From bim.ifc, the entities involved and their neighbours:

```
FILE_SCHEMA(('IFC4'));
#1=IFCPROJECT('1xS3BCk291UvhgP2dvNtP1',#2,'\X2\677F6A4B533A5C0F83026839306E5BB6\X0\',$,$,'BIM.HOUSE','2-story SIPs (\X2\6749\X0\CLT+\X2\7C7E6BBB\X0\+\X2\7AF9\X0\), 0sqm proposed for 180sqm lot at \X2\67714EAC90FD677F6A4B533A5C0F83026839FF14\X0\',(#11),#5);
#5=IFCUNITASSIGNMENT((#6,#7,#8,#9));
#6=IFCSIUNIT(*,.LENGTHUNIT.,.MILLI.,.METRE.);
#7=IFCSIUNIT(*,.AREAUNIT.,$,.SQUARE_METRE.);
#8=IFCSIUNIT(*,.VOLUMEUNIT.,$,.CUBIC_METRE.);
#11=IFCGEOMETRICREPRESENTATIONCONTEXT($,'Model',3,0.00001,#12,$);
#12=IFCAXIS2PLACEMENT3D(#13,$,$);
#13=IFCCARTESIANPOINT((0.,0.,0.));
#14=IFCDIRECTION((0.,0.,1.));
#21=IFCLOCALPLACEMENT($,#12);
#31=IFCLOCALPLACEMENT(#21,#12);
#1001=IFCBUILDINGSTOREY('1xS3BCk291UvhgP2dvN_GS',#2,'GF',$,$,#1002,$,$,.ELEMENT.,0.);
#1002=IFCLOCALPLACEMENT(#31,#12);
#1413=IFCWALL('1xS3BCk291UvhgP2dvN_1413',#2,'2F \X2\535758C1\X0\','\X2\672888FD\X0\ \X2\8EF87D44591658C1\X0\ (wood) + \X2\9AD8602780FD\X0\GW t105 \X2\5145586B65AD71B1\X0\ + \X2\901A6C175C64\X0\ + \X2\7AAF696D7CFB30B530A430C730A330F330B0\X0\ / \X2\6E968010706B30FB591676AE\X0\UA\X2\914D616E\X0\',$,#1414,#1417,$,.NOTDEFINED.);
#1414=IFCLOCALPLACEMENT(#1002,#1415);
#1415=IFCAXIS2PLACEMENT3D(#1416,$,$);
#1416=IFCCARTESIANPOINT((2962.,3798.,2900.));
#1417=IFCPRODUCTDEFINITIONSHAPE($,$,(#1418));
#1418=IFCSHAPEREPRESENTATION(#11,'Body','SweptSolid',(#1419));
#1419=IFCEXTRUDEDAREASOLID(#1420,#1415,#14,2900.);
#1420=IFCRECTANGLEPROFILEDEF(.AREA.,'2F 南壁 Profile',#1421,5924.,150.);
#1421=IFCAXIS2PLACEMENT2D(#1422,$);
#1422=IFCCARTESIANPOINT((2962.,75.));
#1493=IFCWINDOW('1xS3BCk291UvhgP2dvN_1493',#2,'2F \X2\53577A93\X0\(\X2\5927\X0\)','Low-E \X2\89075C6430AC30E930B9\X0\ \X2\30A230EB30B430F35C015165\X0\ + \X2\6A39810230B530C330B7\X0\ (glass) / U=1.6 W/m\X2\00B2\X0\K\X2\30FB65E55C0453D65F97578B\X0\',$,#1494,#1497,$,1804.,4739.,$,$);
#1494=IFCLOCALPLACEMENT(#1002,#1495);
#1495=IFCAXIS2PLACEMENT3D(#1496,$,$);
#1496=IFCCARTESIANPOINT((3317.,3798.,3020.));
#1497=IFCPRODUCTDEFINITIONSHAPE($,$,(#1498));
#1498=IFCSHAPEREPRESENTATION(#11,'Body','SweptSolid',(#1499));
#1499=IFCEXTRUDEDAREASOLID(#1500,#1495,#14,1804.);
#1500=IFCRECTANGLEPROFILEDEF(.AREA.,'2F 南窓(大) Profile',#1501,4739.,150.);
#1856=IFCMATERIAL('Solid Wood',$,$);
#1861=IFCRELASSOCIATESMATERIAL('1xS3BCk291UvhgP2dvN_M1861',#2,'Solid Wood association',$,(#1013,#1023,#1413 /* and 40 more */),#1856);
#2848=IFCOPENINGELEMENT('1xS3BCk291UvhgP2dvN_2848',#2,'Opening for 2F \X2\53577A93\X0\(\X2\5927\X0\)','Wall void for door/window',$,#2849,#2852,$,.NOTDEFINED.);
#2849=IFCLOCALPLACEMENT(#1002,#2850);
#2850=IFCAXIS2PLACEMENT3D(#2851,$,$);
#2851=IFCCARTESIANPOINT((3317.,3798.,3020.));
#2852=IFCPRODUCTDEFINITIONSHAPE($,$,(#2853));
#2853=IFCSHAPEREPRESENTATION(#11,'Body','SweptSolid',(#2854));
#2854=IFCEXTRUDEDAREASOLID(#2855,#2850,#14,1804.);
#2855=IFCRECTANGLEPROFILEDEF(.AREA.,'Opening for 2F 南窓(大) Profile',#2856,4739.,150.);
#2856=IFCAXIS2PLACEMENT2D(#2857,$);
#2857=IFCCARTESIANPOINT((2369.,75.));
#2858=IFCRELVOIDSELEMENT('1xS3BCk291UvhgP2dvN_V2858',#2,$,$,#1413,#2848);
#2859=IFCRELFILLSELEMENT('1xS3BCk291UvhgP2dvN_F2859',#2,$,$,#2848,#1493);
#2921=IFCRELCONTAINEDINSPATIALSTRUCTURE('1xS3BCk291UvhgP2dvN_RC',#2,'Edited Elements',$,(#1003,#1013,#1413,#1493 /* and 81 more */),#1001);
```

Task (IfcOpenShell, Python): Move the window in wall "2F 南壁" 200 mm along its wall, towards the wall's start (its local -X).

```python
import ifcopenshell
import ifcopenshell.api.geometry
import ifcopenshell.util.placement

model = ifcopenshell.open("bim.ifc")

window = model.by_guid("1xS3BCk291UvhgP2dvN_1493")
opening = window.FillsVoids[0].RelatingOpeningElement
wall = opening.VoidsElements[0].RelatingBuildingElement

wall_matrix = ifcopenshell.util.placement.get_local_placement(wall.ObjectPlacement)
shift = wall_matrix[:3, 0] * -200.0
before = ifcopenshell.util.placement.get_local_placement(window.ObjectPlacement)[:3, 3].copy()

# The window is not placed relative to its opening, so move both.
for product in (opening, window):
    matrix = ifcopenshell.util.placement.get_local_placement(product.ObjectPlacement)
    matrix[:3, 3] += shift
    ifcopenshell.api.geometry.edit_object_placement(model, product=product, matrix=matrix, is_si=False)

after = ifcopenshell.util.placement.get_local_placement(window.ObjectPlacement)[:3, 3]
print("window moved by", (after - before).round(3) + 0.0)

model.write("bim-out.ifc")
```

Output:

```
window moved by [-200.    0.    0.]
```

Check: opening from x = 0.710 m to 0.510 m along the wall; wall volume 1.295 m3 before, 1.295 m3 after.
